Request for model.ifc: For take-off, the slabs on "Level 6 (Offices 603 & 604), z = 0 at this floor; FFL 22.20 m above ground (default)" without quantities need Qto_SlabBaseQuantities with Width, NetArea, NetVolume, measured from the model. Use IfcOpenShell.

First a look at what the model holds.

```python
import ifcopenshell
import ifcopenshell.util.element
import ifcopenshell.util.unit

model = ifcopenshell.open("model.ifc")
print(model.schema)
for unit_type in ("LENGTHUNIT", "AREAUNIT", "VOLUMEUNIT"):
    print(unit_type, ifcopenshell.util.unit.calculate_unit_scale(model, unit_type))
storey = next(s for s in model.by_type("IfcBuildingStorey") if s.Name == "Level 6 (Offices 603 & 604), z = 0 at this floor; FFL 22.20 m above ground (default)")
slabs = [e for e in ifcopenshell.util.element.get_decomposition(storey) if e.is_a("IfcSlab")]
for e in sorted(slabs, key=lambda e: e.id()):
    print(e.id(), e.is_a(), e.Name, list(ifcopenshell.util.element.get_psets(e, qtos_only=True)), sep=" | ")
```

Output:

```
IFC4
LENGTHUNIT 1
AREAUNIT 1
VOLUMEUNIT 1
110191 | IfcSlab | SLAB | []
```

```python
import ifcopenshell
import ifcopenshell.api.pset
import ifcopenshell.geom
import ifcopenshell.util.element
import ifcopenshell.util.shape
import ifcopenshell.util.unit

model = ifcopenshell.open("model.ifc")
unit_scale = ifcopenshell.util.unit.calculate_unit_scale(model)
area_scale = ifcopenshell.util.unit.calculate_unit_scale(model, "AREAUNIT")
volume_scale = ifcopenshell.util.unit.calculate_unit_scale(model, "VOLUMEUNIT")
settings = ifcopenshell.geom.settings()

storey = next(s for s in model.by_type("IfcBuildingStorey") if s.Name == "Level 6 (Offices 603 & 604), z = 0 at this floor; FFL 22.20 m above ground (default)")
slabs = [e for e in ifcopenshell.util.element.get_decomposition(storey) if e.is_a("IfcSlab")]

for e in sorted(slabs, key=lambda e: e.id()):
    if ifcopenshell.util.element.get_psets(e, qtos_only=True, should_inherit=False):
        continue
    # Geometry comes back in metres, in the element's own axes.
    shape = ifcopenshell.geom.create_shape(settings, e)
    values = {
        "Width": ifcopenshell.util.shape.get_z(shape.geometry) / unit_scale,
        "NetArea": ifcopenshell.util.shape.get_footprint_area(shape.geometry) / area_scale,
        "NetVolume": ifcopenshell.util.shape.get_volume(shape.geometry) / volume_scale,
    }
    qto = ifcopenshell.api.pset.add_qto(model, product=e, name="Qto_SlabBaseQuantities")
    ifcopenshell.api.pset.edit_qto(model, qto=qto, properties=values)
    print(e.id(), {k: round(v, 3) for k, v in values.items()})

model.write("model-out.ifc")
```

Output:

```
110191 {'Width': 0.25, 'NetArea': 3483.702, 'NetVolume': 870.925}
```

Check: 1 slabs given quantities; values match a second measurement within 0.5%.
